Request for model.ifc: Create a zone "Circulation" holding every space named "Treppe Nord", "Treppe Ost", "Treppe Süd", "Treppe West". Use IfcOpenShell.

First a look at what the model holds.

```python
import ifcopenshell

model = ifcopenshell.open("model.ifc")
print(model.schema)
seen = {}
for space in model.by_type("IfcSpace"):
    seen[space.LongName] = seen.get(space.LongName, 0) + 1
for name, count in sorted(seen.items(), key=str):
    print(count, "x", name)
print("zones:", [z.Name for z in model.by_type("IfcZone")][:20])
```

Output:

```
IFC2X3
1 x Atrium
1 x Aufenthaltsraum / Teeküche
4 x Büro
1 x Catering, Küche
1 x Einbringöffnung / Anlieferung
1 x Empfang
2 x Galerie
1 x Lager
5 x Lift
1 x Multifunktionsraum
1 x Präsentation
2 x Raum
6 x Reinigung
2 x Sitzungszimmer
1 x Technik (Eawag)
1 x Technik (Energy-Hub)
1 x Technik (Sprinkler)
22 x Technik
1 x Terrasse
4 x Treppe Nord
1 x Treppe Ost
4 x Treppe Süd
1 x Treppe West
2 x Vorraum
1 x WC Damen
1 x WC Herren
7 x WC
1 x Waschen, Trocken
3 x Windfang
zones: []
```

```python
import ifcopenshell
import ifcopenshell.api.group
import ifcopenshell.api.root

model = ifcopenshell.open("model.ifc")

names = {"Treppe Nord", "Treppe Ost", "Treppe Süd", "Treppe West"}
spaces = [s for s in model.by_type("IfcSpace") if s.LongName in names]

zone = ifcopenshell.api.root.create_entity(model, ifc_class="IfcZone", name="Circulation")
ifcopenshell.api.group.assign_group(model, products=spaces, group=zone)
print(len(spaces), "spaces in", zone.Name)

model.write("model-out.ifc")
```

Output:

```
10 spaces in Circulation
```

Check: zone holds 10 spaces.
